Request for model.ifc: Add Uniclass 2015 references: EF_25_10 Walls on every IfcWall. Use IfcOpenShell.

First a look at what the model holds.

```python
import ifcopenshell

model = ifcopenshell.open("model.ifc")
print(model.schema)
print("classifications:", [c.Name for c in model.by_type("IfcClassification")])
for ifc_class in ("IfcDoor", "IfcRoof", "IfcStair", "IfcWall", "IfcWindow"):
    print(ifc_class, len(model.by_type(ifc_class)))
```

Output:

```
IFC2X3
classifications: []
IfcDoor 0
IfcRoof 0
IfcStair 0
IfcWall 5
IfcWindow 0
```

```python
import ifcopenshell
import ifcopenshell.api.classification

model = ifcopenshell.open("model.ifc")

# IFC2X3 requires Source and Edition and has no link from the project to the system.
system = model.create_entity("IfcClassification", Source="NBS", Edition="2015", Name="Uniclass 2015")

codes = {
    "IfcWall": ("EF_25_10", "Walls"),
}
for ifc_class, (code, name) in codes.items():
    products = model.by_type(ifc_class)
    ifcopenshell.api.classification.add_reference(
        model, products=products, classification=system, identification=code, name=name
    )
    print(code, len(products))

model.write("model-out.ifc")
```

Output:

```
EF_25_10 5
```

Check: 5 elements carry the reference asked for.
